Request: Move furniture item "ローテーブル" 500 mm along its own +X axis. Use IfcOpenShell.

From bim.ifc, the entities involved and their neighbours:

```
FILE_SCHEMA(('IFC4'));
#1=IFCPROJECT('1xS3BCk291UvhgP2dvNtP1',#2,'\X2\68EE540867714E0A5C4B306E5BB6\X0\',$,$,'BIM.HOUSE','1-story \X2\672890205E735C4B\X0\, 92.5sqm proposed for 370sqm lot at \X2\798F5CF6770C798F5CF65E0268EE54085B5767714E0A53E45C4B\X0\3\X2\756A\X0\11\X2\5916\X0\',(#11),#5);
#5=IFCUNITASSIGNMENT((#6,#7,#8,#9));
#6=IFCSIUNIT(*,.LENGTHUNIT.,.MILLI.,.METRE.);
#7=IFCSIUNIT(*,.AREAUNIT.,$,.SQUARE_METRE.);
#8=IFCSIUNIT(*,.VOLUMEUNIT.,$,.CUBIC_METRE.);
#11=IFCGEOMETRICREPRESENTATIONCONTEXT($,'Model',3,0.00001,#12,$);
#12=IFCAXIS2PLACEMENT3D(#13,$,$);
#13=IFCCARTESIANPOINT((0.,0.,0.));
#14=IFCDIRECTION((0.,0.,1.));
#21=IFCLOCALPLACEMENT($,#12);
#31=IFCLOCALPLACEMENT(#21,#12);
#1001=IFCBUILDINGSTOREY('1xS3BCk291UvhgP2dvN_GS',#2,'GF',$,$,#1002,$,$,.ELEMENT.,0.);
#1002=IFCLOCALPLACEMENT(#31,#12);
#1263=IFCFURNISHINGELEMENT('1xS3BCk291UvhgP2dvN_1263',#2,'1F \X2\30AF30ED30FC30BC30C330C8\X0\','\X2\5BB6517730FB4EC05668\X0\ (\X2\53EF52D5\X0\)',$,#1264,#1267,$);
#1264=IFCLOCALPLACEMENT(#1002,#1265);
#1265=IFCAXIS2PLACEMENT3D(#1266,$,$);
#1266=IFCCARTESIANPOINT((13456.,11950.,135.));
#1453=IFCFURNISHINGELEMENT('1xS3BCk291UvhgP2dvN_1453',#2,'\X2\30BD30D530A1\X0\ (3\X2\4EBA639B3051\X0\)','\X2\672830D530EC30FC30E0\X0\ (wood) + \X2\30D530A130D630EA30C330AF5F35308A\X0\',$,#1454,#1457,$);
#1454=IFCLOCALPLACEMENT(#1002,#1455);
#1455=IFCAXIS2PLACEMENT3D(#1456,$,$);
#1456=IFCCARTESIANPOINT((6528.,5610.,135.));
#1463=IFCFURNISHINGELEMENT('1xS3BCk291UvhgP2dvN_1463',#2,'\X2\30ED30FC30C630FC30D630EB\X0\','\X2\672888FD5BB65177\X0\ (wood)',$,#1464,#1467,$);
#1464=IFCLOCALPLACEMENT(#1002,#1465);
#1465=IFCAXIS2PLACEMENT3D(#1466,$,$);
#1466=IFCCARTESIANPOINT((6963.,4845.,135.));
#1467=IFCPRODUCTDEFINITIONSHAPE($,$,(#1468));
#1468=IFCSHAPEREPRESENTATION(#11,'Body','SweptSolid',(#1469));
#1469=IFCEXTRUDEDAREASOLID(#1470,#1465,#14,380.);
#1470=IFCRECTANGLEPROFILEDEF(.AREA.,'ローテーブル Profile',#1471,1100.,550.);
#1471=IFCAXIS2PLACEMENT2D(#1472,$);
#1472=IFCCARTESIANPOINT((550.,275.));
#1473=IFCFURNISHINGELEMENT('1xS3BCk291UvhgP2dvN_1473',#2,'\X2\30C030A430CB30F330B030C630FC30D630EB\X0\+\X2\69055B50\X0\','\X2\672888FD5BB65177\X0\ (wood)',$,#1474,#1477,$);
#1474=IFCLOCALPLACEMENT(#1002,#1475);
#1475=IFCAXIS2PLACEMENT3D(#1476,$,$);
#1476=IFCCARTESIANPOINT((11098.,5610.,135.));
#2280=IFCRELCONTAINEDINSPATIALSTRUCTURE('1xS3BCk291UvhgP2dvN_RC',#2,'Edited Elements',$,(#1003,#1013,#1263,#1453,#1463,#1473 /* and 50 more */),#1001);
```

```python
import ifcopenshell
import ifcopenshell.api.geometry
import ifcopenshell.util.placement

model = ifcopenshell.open("bim.ifc")

item = model.by_id(1463)
matrix = ifcopenshell.util.placement.get_local_placement(item.ObjectPlacement)
matrix[:3, 3] += matrix[:3, 0] * 500.0
ifcopenshell.api.geometry.edit_object_placement(model, product=item, matrix=matrix, is_si=False)

print(ifcopenshell.util.placement.get_local_placement(item.ObjectPlacement).round(3) + 0.0)

model.write("bim_edited.ifc")
```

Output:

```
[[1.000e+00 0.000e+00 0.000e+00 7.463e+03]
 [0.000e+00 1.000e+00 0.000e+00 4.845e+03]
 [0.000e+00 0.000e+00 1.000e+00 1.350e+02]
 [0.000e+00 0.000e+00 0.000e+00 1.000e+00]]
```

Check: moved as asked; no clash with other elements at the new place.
